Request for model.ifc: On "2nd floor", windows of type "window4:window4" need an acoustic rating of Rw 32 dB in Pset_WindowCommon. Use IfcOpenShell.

First a look at what the model holds.

```python
import ifcopenshell
import ifcopenshell.util.element

model = ifcopenshell.open("model.ifc")
print(model.schema)
storey = next(s for s in model.by_type("IfcBuildingStorey") if s.Name == "2nd floor")
windows = [e for e in ifcopenshell.util.element.get_decomposition(storey) if e.is_a("IfcWindow")]
seen = {}
for e in windows:
    element_type = ifcopenshell.util.element.get_type(e)
    key = (element_type.Name if element_type != e and element_type else None, ifcopenshell.util.element.get_pset(e, "Pset_WindowCommon", "AcousticRating"))
    seen[key] = seen.get(key, 0) + 1
for (name, value), count in sorted(seen.items(), key=str):
    print(count, "x", name, "|", value)
```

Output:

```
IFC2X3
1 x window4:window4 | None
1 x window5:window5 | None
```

```python
import ifcopenshell
import ifcopenshell.api.pset
import ifcopenshell.util.element

model = ifcopenshell.open("model.ifc")

storey = next(s for s in model.by_type("IfcBuildingStorey") if s.Name == "2nd floor")
windows = [e for e in ifcopenshell.util.element.get_decomposition(storey) if e.is_a("IfcWindow")]

count = 0
for e in windows:
    element_type = ifcopenshell.util.element.get_type(e)
    if element_type in (None, e) or element_type.Name != "window4:window4":
        continue
    # add_pset returns the element's existing set when there is one.
    pset = ifcopenshell.api.pset.add_pset(model, product=e, name="Pset_WindowCommon")
    ifcopenshell.api.pset.edit_pset(model, pset=pset, properties={"AcousticRating": "Rw 32 dB"})
    count += 1

print(count, "windows updated")

model.write("model-out.ifc")
```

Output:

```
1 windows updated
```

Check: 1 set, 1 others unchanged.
